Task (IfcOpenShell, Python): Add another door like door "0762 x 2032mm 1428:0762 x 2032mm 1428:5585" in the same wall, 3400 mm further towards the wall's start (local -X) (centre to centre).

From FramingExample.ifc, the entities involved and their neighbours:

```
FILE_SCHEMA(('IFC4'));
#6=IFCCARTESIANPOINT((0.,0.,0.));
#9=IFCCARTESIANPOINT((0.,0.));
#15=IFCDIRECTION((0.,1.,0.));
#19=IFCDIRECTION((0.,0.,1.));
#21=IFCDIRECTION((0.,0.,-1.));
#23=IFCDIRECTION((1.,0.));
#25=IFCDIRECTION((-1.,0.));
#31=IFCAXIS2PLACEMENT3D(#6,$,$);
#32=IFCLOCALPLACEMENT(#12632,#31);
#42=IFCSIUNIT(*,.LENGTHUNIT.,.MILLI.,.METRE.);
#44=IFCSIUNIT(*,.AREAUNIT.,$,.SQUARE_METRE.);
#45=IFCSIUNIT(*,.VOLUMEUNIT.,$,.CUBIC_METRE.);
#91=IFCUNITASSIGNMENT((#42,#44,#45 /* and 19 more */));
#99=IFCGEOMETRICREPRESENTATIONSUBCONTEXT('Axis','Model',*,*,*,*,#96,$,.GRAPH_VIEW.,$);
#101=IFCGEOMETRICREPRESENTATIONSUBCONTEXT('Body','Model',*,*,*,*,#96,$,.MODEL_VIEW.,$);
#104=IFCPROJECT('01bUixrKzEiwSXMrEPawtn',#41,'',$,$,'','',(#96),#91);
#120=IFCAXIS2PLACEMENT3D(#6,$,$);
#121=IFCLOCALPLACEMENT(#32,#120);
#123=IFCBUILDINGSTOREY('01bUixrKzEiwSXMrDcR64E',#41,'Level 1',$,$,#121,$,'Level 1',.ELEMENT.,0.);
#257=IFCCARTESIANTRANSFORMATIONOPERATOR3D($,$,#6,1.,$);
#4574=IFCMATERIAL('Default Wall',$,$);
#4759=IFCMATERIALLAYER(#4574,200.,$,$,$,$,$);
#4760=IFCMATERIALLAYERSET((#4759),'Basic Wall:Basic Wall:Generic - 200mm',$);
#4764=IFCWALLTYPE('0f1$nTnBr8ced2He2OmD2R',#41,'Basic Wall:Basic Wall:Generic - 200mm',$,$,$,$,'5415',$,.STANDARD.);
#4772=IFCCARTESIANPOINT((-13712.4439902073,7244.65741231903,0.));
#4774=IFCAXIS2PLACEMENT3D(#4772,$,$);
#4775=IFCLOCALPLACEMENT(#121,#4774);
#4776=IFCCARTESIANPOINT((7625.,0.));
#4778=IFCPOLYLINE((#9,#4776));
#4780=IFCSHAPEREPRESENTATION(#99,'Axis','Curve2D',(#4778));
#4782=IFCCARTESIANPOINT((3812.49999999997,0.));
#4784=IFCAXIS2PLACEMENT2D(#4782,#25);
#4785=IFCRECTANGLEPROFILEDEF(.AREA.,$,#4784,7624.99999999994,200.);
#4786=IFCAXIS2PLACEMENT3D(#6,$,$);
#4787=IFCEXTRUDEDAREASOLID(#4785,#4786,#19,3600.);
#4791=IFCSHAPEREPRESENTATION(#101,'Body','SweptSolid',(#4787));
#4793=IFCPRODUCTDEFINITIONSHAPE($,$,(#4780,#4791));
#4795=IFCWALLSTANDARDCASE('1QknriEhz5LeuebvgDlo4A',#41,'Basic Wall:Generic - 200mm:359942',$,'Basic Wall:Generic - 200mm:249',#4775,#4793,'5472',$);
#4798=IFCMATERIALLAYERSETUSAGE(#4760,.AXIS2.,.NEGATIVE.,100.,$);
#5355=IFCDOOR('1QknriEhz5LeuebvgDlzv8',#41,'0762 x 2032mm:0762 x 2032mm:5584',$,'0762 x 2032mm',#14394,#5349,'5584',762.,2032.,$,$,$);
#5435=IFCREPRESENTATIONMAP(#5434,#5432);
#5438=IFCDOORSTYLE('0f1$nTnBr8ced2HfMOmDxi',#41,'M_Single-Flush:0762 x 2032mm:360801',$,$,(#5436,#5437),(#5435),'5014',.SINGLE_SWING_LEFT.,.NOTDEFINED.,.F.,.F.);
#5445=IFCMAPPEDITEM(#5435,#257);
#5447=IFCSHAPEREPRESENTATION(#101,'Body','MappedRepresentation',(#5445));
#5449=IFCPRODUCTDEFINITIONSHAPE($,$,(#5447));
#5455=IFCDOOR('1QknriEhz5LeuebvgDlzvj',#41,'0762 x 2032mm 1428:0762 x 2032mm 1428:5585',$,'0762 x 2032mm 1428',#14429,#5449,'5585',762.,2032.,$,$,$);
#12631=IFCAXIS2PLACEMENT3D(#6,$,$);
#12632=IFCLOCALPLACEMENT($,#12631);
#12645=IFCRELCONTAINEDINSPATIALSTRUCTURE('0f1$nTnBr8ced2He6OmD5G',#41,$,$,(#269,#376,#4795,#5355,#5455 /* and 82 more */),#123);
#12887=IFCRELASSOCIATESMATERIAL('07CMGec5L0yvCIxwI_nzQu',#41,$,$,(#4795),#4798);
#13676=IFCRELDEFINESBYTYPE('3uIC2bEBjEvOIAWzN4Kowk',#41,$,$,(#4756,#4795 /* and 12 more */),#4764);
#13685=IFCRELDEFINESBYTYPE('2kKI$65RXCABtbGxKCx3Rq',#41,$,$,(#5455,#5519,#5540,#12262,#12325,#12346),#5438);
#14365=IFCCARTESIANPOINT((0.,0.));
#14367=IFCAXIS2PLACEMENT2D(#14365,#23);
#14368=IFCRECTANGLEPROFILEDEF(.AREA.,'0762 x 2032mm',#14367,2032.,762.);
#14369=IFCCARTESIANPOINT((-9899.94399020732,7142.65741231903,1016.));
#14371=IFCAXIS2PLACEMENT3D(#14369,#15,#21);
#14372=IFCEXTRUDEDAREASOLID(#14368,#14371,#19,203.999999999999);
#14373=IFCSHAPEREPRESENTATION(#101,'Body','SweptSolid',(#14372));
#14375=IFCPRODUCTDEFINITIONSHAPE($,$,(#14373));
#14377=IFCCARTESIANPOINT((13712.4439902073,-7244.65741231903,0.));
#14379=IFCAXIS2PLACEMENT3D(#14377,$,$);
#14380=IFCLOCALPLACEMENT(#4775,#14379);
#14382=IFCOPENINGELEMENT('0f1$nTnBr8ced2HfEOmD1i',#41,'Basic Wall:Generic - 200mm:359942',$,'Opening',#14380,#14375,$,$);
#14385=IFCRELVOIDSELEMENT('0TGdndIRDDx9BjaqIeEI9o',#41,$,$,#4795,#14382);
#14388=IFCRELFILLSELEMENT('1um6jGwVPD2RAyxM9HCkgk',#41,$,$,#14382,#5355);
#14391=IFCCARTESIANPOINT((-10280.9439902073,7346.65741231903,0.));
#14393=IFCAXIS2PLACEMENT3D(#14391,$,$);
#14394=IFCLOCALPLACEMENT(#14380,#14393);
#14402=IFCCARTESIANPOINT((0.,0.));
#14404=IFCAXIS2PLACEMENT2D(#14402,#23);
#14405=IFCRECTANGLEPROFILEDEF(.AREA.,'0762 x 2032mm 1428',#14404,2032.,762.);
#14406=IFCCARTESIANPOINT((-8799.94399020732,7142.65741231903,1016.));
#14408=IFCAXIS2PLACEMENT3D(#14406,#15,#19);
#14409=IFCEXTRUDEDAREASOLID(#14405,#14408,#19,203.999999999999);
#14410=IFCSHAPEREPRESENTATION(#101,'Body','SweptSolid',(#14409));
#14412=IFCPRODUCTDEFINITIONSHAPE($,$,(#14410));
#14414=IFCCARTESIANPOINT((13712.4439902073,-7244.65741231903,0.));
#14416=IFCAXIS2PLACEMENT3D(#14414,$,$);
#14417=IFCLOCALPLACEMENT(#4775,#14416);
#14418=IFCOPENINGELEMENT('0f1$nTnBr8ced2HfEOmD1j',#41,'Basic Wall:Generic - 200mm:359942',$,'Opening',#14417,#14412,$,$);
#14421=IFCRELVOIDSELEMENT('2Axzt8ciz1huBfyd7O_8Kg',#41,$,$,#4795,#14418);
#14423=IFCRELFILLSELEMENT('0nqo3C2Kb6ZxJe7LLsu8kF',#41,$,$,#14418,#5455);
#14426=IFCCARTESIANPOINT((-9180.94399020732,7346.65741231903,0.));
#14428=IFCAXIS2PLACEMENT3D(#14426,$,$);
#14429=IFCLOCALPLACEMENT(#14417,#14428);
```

```python
import ifcopenshell
import ifcopenshell.api.feature
import ifcopenshell.api.geometry
import ifcopenshell.api.root
import ifcopenshell.geom
import ifcopenshell.util.element
import ifcopenshell.util.placement
import ifcopenshell.util.shape

model = ifcopenshell.open("FramingExample.ifc")
settings = ifcopenshell.geom.settings()


def volume(element):
    """Net volume in cubic metres, openings subtracted."""
    shape = ifcopenshell.geom.create_shape(settings, element)
    return ifcopenshell.util.shape.get_volume(shape.geometry)


def reuse_history(source, copy):
    """copy_class also copies each property set's owner history, people and application; keep the originals."""
    for rel in copy.IsDefinedBy:
        if rel.is_a("IfcRelDefinesByProperties") and (history := rel.RelatingPropertyDefinition.OwnerHistory):
            rel.RelatingPropertyDefinition.OwnerHistory = source.OwnerHistory
            ifcopenshell.util.element.remove_deep2(model, history)


door = model.by_guid("1QknriEhz5LeuebvgDlzvj")
opening = door.FillsVoids[0].RelatingOpeningElement
wall = opening.VoidsElements[0].RelatingBuildingElement
before = volume(wall)
shift = ifcopenshell.util.placement.get_local_placement(wall.ObjectPlacement)[:3, 0] * -3400.0

# copy_class copies the void relationship, type, container and properties, but no geometry.
new_opening = ifcopenshell.api.root.copy_class(model, product=opening)
new_opening.Representation = ifcopenshell.util.element.copy_deep(
    model, opening.Representation, exclude=["IfcGeometricRepresentationContext", "IfcRepresentationMap"]
)
new_opening.Name = "Basic Wall:Generic - 200mm"
new_door = ifcopenshell.api.root.copy_class(model, product=door)
new_door.Representation = ifcopenshell.util.element.copy_deep(
    model, door.Representation, exclude=["IfcGeometricRepresentationContext", "IfcRepresentationMap"]
)
new_door.Name = "0762 x 2032mm 1428:0762 x 2032mm 1428"
new_door.Tag = None
reuse_history(door, new_door)
ifcopenshell.api.feature.add_filling(model, opening=new_opening, element=new_door)

for old, new in ((opening, new_opening), (door, new_door)):
    matrix = ifcopenshell.util.placement.get_local_placement(old.ObjectPlacement)
    matrix[:3, 3] += shift
    ifcopenshell.api.geometry.edit_object_placement(model, product=new, matrix=matrix, is_si=False)

after = volume(wall)

print(f"wall volume {before:.3f} -> {after:.3f} m3")

model.write("FramingExample_updated.ifc")
```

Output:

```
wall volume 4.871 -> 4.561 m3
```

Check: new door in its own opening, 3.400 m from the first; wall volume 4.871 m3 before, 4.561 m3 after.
